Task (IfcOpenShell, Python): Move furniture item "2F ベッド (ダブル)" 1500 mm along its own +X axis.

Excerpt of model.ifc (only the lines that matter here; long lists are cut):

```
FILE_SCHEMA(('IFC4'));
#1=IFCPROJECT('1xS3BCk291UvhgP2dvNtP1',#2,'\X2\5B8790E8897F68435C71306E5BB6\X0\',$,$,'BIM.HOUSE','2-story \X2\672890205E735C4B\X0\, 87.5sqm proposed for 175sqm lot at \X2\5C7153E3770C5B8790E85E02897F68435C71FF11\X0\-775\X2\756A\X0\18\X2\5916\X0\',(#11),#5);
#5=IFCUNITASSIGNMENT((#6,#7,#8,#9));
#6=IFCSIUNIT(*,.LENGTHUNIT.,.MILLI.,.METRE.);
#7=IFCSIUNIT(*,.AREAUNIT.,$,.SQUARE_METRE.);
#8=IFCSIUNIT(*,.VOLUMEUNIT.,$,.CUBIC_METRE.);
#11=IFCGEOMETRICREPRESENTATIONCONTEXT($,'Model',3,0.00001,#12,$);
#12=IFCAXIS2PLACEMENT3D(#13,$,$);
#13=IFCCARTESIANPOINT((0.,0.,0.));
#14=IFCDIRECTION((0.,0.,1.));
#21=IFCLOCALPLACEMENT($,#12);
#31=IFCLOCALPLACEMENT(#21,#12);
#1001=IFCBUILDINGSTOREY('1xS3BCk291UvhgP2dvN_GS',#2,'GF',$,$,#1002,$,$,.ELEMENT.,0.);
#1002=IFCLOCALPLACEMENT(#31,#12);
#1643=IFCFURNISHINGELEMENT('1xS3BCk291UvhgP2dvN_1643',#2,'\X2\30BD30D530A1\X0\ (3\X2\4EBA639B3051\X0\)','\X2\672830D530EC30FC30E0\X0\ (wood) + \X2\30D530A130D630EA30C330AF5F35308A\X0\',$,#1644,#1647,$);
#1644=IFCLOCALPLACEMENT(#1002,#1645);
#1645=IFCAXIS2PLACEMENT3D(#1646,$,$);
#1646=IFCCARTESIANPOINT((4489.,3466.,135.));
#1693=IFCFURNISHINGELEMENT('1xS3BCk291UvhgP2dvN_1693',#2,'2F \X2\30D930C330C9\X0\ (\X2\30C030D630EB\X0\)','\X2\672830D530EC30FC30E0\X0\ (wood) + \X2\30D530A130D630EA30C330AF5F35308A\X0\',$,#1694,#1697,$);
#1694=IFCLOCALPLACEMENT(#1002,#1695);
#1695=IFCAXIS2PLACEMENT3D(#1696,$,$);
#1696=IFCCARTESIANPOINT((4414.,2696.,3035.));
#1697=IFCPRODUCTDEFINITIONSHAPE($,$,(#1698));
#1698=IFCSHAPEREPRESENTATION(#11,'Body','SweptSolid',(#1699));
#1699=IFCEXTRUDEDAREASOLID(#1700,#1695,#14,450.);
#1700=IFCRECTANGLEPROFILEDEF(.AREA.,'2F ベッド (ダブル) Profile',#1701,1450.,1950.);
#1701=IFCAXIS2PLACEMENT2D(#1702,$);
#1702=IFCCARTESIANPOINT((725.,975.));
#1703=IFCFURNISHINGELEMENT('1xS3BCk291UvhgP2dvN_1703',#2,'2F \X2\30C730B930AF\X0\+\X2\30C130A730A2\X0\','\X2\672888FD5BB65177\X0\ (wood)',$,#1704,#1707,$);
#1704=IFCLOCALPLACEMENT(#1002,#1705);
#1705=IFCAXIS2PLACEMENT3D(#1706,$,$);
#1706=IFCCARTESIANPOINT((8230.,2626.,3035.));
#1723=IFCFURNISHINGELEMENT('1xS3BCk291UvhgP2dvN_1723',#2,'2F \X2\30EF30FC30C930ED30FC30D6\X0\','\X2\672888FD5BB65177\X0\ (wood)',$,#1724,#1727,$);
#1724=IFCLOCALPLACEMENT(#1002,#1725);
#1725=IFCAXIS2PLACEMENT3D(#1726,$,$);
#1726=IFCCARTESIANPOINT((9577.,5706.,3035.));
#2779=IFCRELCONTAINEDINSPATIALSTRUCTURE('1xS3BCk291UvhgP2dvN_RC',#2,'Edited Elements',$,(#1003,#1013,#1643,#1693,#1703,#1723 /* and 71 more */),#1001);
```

```python
import ifcopenshell
import ifcopenshell.api.geometry
import ifcopenshell.util.placement
import ifcopenshell.util.unit

model = ifcopenshell.open("model.ifc")
unit_scale = ifcopenshell.util.unit.calculate_unit_scale(model)

item = model.by_guid("1xS3BCk291UvhgP2dvN_1693")
matrix = ifcopenshell.util.placement.get_local_placement(item.ObjectPlacement)
matrix[:3, 3] += matrix[:3, 0] * 1.5 / unit_scale
ifcopenshell.api.geometry.edit_object_placement(model, product=item, matrix=matrix, is_si=False)

print(ifcopenshell.util.placement.get_local_placement(item.ObjectPlacement).round(3) + 0.0)

model.write("model_rev.ifc")
```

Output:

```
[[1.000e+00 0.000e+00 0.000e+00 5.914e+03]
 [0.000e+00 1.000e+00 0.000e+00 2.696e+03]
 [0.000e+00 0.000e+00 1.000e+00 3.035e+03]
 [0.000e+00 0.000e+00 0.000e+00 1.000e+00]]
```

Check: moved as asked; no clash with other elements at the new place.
